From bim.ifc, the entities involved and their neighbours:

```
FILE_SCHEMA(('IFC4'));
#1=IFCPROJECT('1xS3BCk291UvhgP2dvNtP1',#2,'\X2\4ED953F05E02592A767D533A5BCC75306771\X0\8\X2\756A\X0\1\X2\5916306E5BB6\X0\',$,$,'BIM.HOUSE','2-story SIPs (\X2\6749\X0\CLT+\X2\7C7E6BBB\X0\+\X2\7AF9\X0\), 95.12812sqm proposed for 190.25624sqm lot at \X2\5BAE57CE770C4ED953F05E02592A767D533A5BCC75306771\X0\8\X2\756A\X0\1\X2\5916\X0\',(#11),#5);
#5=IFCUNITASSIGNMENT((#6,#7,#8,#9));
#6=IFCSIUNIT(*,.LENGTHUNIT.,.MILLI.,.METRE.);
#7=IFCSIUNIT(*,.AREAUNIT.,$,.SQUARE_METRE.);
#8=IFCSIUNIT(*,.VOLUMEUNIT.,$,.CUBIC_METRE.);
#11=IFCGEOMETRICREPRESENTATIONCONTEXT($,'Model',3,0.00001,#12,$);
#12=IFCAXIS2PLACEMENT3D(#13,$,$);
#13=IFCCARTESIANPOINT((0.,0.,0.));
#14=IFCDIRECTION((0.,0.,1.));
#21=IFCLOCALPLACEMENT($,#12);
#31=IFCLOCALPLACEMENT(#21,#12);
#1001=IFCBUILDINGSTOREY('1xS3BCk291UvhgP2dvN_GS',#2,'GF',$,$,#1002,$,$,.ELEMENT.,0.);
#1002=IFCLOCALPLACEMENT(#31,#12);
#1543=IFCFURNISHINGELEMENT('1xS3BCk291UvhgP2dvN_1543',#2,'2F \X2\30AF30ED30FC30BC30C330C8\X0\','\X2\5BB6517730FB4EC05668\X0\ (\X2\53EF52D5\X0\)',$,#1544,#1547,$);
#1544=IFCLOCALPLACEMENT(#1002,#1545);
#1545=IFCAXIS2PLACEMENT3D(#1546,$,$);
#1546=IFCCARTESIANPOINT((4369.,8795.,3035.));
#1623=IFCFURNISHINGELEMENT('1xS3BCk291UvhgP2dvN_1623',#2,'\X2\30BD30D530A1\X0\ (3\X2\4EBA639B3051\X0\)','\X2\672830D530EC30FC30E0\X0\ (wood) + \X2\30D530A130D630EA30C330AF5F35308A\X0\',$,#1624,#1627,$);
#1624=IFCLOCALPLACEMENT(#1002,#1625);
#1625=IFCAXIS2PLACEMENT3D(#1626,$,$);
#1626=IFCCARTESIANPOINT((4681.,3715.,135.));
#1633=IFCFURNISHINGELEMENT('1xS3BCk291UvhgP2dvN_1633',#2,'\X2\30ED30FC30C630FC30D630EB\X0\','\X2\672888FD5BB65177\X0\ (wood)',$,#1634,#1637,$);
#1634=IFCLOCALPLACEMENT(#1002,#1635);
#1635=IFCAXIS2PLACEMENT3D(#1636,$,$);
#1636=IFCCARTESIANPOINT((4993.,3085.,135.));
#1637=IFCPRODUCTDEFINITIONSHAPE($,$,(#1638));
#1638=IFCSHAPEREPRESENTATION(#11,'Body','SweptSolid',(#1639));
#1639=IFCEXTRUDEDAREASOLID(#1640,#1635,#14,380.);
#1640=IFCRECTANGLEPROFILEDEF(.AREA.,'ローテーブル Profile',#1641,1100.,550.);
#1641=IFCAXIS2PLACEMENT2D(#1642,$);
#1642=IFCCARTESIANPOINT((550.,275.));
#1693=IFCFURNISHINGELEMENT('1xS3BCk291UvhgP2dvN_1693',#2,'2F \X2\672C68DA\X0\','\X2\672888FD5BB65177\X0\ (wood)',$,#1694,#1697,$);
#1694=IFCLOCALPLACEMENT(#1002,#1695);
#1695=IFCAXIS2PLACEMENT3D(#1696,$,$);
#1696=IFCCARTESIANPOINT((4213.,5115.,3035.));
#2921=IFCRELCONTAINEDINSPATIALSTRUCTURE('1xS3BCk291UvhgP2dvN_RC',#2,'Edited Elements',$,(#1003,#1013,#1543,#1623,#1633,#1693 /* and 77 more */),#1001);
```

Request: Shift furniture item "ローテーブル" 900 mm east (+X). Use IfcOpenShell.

```python
import ifcopenshell
import ifcopenshell.api.geometry
import ifcopenshell.util.placement
import ifcopenshell.util.unit

model = ifcopenshell.open("bim.ifc")
unit_scale = ifcopenshell.util.unit.calculate_unit_scale(model)

item = model.by_guid("1xS3BCk291UvhgP2dvN_1633")
matrix = ifcopenshell.util.placement.get_local_placement(item.ObjectPlacement)
matrix[0, 3] += 0.9 / unit_scale
ifcopenshell.api.geometry.edit_object_placement(model, product=item, matrix=matrix, is_si=False)

print(ifcopenshell.util.placement.get_local_placement(item.ObjectPlacement).round(3) + 0.0)

model.write("bim_v2.ifc")
```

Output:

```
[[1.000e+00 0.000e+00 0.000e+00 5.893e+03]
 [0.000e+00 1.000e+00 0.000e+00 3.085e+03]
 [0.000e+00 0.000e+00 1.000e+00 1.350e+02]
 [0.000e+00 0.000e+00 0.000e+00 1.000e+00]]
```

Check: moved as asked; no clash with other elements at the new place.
